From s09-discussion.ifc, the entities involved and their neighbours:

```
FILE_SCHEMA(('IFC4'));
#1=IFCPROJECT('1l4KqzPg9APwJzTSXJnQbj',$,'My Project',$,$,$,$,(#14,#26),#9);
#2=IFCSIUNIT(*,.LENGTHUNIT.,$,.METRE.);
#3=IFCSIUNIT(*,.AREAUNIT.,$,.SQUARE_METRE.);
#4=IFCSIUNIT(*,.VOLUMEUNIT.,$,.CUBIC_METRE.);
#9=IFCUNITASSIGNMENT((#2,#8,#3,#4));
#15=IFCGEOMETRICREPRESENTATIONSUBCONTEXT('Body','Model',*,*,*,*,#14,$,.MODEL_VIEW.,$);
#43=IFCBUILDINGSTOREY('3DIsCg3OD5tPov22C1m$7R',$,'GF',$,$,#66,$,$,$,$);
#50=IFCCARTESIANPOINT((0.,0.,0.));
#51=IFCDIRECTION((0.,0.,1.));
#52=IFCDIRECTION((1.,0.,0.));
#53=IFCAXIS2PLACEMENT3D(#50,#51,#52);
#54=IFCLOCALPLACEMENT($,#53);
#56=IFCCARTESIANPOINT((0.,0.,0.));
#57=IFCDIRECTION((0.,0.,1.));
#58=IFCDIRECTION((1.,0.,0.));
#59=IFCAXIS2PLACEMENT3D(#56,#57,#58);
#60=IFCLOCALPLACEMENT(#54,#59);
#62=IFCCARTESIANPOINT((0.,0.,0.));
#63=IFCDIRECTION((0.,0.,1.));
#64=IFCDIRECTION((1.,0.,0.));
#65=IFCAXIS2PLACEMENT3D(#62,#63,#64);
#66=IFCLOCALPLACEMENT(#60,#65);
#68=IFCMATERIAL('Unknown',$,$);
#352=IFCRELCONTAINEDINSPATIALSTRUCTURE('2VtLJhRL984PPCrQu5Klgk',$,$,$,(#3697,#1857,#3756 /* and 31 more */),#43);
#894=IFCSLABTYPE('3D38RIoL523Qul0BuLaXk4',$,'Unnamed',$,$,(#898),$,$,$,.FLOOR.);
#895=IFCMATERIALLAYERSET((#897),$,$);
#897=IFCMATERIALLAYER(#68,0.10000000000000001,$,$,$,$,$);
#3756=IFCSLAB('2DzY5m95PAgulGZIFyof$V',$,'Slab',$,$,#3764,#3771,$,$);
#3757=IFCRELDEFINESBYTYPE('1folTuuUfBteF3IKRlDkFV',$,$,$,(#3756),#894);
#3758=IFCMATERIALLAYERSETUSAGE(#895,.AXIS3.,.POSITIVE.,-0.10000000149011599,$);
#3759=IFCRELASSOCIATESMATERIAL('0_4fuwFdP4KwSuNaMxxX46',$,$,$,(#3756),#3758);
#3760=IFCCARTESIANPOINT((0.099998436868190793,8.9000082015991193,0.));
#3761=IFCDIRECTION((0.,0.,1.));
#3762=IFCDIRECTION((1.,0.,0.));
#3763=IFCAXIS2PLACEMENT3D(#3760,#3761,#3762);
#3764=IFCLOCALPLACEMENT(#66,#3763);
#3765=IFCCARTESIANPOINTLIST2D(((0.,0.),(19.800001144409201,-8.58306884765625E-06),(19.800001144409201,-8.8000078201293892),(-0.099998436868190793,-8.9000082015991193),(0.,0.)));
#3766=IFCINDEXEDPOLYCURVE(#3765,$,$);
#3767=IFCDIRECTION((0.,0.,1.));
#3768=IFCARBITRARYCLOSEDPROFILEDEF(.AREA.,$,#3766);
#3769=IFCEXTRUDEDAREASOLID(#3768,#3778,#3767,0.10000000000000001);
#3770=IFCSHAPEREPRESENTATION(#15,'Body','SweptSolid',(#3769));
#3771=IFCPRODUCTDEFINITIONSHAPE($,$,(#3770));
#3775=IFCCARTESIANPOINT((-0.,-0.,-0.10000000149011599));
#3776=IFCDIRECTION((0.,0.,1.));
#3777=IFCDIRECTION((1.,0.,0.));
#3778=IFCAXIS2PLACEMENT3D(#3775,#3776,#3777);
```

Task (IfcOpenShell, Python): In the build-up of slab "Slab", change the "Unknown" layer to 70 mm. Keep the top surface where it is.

```python
import ifcopenshell
import ifcopenshell.util.element
import ifcopenshell.util.representation
import ifcopenshell.util.unit

model = ifcopenshell.open("s09-discussion.ifc")
unit_scale = ifcopenshell.util.unit.calculate_unit_scale(model)

layer_set = model.by_id(895)
layer = next(l for l in layer_set.MaterialLayers if l.Material and l.Material.Name == "Unknown")
change = 0.07 / unit_scale - layer.LayerThickness
layer.LayerThickness += change

# Geometry does not follow the layer set by itself.
slabs = [e for e in ifcopenshell.util.element.get_elements_by_material(model, layer_set) if e.is_a("IfcSlab")]
for slab in sorted(slabs, key=lambda e: e.id()):
    body = ifcopenshell.util.representation.get_representation(slab, "Model", "Body")
    solid = body.Items[0]
    old_depth = solid.Depth
    solid.Depth += change
    # Extruded upwards: lower the start of the extrusion so the top stays.
    x, y, z = solid.Position.Location.Coordinates
    solid.Position.Location = model.createIfcCartesianPoint((x, y, z - change))
    print(slab.id(), f"{old_depth:g} -> {solid.Depth:g}")

# The layers are counted up from the underside, which has moved.
for usage in {ifcopenshell.util.element.get_material(slab) for slab in slabs}:
    usage.OffsetFromReferenceLine -= change

model.write("s09-discussion_rev.ifc")
```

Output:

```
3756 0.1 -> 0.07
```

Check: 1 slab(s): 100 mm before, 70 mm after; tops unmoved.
